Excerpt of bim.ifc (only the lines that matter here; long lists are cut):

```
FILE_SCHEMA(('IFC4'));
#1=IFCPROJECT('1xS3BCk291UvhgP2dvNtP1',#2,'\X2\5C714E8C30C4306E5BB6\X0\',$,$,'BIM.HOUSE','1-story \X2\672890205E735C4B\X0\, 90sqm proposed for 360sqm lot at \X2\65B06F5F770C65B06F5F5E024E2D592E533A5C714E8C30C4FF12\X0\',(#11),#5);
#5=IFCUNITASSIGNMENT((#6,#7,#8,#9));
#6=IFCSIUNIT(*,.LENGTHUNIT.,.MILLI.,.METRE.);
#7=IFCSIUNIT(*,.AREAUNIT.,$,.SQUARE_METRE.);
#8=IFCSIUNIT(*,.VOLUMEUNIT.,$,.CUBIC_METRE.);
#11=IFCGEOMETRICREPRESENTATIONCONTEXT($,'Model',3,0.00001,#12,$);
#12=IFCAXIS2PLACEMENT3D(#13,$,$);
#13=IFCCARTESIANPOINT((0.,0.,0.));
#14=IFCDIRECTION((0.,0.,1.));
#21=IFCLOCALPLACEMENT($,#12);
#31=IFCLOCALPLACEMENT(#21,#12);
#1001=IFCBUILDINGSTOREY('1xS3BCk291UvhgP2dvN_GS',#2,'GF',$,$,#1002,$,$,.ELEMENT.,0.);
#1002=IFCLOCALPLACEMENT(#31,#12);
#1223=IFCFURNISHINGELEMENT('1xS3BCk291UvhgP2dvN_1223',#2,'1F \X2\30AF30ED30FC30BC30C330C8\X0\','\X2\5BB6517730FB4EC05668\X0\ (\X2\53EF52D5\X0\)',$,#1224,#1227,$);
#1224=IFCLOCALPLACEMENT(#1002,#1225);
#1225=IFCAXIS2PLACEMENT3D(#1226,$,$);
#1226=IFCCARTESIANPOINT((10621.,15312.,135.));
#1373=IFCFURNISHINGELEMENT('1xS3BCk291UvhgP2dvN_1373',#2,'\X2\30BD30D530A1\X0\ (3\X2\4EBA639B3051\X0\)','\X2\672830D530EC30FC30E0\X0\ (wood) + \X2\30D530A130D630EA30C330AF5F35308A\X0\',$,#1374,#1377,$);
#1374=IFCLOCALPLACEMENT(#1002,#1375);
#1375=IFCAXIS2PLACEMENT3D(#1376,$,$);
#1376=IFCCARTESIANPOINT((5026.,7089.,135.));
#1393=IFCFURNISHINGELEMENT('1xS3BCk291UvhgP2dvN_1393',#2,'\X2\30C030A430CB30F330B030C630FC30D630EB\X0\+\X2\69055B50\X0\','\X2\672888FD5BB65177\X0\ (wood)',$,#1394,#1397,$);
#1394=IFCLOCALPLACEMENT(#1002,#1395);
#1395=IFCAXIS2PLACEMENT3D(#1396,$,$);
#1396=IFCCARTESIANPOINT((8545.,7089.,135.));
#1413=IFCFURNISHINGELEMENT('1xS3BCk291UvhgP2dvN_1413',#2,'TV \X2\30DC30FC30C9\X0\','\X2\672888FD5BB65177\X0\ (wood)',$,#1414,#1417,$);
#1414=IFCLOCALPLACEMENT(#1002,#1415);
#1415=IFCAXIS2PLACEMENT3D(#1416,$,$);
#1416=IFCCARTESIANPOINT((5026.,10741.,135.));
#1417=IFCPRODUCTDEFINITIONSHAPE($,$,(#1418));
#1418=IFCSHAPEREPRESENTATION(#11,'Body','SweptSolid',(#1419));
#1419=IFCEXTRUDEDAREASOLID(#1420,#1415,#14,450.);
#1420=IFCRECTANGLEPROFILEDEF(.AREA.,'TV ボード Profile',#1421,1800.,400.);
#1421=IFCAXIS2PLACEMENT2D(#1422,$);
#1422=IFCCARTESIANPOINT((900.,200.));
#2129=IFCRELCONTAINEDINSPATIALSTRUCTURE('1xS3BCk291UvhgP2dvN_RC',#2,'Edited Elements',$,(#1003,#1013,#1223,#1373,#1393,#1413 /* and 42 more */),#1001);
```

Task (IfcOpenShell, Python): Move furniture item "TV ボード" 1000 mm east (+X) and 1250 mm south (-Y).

```python
import ifcopenshell
import ifcopenshell.api.geometry
import ifcopenshell.util.placement

model = ifcopenshell.open("bim.ifc")

item = model.by_guid("1xS3BCk291UvhgP2dvN_1413")
matrix = ifcopenshell.util.placement.get_local_placement(item.ObjectPlacement)
matrix[0, 3] += 1000.0
matrix[1, 3] -= 1250.0
ifcopenshell.api.geometry.edit_object_placement(model, product=item, matrix=matrix, is_si=False)

print(ifcopenshell.util.placement.get_local_placement(item.ObjectPlacement).round(3) + 0.0)

model.write("bim-out.ifc")
```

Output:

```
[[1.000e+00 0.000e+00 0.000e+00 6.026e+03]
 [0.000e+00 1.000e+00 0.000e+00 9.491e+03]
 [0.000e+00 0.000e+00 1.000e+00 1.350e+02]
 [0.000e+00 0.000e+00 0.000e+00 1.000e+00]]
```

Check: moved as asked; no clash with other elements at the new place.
